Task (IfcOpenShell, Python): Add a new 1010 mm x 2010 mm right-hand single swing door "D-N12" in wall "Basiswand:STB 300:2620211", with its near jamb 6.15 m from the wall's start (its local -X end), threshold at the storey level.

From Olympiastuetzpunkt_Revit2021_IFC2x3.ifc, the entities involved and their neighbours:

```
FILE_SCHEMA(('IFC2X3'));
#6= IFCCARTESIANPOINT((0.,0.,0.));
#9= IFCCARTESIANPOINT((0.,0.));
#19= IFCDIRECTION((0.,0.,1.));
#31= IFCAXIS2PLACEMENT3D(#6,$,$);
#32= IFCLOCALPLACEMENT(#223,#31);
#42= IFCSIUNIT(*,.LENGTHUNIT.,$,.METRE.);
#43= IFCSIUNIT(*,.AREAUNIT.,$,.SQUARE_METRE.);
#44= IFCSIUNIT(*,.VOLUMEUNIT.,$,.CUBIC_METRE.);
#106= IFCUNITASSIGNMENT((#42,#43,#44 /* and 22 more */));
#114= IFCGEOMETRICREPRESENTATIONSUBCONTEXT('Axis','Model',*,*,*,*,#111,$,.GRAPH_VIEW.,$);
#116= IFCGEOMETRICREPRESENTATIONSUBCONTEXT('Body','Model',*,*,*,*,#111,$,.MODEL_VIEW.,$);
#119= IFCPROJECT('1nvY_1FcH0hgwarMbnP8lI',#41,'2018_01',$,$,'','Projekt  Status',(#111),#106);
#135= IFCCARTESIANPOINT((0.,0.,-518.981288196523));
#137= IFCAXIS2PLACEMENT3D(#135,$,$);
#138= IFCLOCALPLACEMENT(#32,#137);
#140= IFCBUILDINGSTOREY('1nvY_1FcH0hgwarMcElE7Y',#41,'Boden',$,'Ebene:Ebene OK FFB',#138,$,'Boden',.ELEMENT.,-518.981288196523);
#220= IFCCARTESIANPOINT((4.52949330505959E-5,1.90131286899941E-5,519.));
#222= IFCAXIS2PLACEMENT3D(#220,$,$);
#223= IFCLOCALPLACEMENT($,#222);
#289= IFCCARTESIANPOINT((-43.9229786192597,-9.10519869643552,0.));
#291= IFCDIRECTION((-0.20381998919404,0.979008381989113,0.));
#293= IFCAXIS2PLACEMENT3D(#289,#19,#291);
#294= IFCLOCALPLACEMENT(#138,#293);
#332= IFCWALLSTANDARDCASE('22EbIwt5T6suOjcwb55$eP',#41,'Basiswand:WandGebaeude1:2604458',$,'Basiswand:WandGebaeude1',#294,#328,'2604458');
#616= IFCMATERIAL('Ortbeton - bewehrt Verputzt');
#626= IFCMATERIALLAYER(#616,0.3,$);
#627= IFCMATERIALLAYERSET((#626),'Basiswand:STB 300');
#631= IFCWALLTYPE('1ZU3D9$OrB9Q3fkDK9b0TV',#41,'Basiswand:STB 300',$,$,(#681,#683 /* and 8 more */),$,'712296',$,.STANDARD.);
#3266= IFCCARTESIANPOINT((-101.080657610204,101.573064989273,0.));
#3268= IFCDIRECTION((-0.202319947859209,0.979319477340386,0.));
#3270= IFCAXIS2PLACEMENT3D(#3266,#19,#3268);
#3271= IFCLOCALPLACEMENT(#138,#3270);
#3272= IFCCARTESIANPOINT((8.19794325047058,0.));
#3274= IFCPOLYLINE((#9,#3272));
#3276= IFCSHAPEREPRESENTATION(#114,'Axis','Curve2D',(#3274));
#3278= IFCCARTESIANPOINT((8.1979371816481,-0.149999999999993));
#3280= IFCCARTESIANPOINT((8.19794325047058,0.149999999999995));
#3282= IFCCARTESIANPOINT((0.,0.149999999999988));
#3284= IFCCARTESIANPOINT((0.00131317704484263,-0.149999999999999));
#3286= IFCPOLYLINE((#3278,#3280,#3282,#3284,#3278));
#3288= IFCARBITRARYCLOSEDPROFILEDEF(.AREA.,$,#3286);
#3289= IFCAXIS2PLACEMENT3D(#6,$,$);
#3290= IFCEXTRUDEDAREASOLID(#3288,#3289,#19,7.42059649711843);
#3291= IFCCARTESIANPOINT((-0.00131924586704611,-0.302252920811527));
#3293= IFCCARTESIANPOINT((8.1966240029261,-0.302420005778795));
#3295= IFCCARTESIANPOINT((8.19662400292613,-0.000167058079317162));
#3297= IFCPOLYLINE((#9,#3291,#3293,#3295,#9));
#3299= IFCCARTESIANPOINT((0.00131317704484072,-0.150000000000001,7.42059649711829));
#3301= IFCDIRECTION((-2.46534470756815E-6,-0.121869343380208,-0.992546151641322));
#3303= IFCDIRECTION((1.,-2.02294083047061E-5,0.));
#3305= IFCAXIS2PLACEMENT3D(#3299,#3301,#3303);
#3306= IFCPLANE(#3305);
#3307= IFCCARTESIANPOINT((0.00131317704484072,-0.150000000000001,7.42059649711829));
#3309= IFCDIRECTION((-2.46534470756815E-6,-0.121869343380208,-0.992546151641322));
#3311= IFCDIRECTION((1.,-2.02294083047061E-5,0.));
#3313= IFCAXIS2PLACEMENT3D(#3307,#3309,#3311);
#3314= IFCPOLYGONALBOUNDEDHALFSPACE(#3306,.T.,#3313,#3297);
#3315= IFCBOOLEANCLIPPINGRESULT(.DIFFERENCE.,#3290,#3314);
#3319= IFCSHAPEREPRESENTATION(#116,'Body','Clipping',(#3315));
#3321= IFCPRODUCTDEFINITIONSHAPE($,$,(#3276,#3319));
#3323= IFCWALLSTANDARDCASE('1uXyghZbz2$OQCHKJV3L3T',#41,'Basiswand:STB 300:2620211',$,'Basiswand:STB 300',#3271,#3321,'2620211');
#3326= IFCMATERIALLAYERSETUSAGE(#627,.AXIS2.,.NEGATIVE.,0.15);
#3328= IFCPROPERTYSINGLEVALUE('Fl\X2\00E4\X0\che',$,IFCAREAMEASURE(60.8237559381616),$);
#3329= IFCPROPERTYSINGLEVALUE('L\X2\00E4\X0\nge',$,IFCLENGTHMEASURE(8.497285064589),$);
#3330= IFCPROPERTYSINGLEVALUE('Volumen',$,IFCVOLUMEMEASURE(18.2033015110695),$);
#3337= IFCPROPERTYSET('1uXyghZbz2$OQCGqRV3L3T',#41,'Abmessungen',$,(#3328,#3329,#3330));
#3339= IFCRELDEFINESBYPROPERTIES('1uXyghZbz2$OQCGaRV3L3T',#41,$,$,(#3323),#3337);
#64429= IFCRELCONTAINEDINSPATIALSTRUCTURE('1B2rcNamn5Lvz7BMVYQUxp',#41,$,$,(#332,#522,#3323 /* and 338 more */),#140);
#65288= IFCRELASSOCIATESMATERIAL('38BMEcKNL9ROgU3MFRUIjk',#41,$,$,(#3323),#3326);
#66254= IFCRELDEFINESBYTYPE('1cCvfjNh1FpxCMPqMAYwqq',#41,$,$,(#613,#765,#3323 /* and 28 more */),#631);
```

```python
import numpy as np
import ifcopenshell
import ifcopenshell.api.feature
import ifcopenshell.api.geometry
import ifcopenshell.api.pset
import ifcopenshell.api.root
import ifcopenshell.api.spatial
import ifcopenshell.api.type
import ifcopenshell.geom
import ifcopenshell.util.element
import ifcopenshell.util.placement
import ifcopenshell.util.representation
import ifcopenshell.util.shape
import ifcopenshell.util.unit

model = ifcopenshell.open("Olympiastuetzpunkt_Revit2021_IFC2x3.ifc")
unit_scale = ifcopenshell.util.unit.calculate_unit_scale(model)
area_scale = ifcopenshell.util.unit.calculate_unit_scale(model, "AREAUNIT")
volume_scale = ifcopenshell.util.unit.calculate_unit_scale(model, "VOLUMEUNIT")
settings = ifcopenshell.geom.settings()


def volume(element):
    """Net volume in cubic metres, openings subtracted."""
    shape = ifcopenshell.geom.create_shape(settings, element)
    return ifcopenshell.util.shape.get_volume(shape.geometry)


wall = model.by_guid("1uXyghZbz2$OQCHKJV3L3T")
storey = ifcopenshell.util.element.get_container(wall, ifc_class="IfcBuildingStorey")
context = ifcopenshell.util.representation.get_context(model, "Model", "Body", "MODEL_VIEW")
before = volume(wall)

width, height, from_end, sill = 1.01, 2.01, 6.15, 0.0  # metres

# The wall runs along its own X axis, and the end named is its -X end.
wall_shape = ifcopenshell.geom.create_shape(settings, wall)
x, y, z = ifcopenshell.util.shape.get_vertices(wall_shape.geometry).T
start = x.min() + from_end
face, thickness = float(y.min()), float(y.max() - y.min())
wall_matrix = ifcopenshell.util.placement.get_local_placement(wall.ObjectPlacement)
level = ifcopenshell.util.placement.get_local_placement(storey.ObjectPlacement)[2, 3]


def in_wall(x, y):
    """Placement at x, y metres in the wall's axes, at sill height."""
    matrix = wall_matrix.copy()
    matrix[:, 3] = wall_matrix @ np.array([x / unit_scale, y / unit_scale, 0.0, 1.0])
    matrix[2, 3] = level + sill / unit_scale
    return matrix


# Opening: a box that overshoots both wall faces by 50 mm.
opening = ifcopenshell.api.root.create_entity(model, ifc_class="IfcOpeningElement")
box = ifcopenshell.api.geometry.add_wall_representation(
    model, context=context, length=width, height=height, thickness=thickness + 0.1
)
ifcopenshell.api.geometry.assign_representation(model, product=opening, representation=box)
ifcopenshell.api.geometry.edit_object_placement(model, product=opening, matrix=in_wall(start, face - 0.05), is_si=False)
ifcopenshell.api.feature.add_feature(model, feature=opening, element=wall)

door = ifcopenshell.api.root.create_entity(model, ifc_class="IfcDoor", name="D-N12")
door.OverallWidth, door.OverallHeight = width / unit_scale, height / unit_scale
body = ifcopenshell.api.geometry.add_door_representation(
    model,
    context=context,
    overall_width=door.OverallWidth,
    overall_height=door.OverallHeight,
    operation_type="SINGLE_SWING_RIGHT",
    lining_properties={"LiningDepth": thickness / unit_scale, "ThresholdDepth": thickness / unit_scale},
)
ifcopenshell.api.geometry.assign_representation(model, product=door, representation=body)
ifcopenshell.api.spatial.assign_container(model, products=[door], relating_structure=storey)
fills = ifcopenshell.api.feature.add_filling(model, opening=opening, element=door)
fills.OwnerHistory = door.OwnerHistory  # required in IFC2X3

# IFC2X3 keeps the operation on the door style.
style = ifcopenshell.api.root.create_entity(model, ifc_class="IfcDoorStyle", name="D-N12")
style.OperationType, style.ConstructionType = "SINGLE_SWING_RIGHT", "NOTDEFINED"
style.ParameterTakesPrecedence = style.Sizeable = False
ifcopenshell.api.type.assign_type(model, related_objects=[door], relating_type=style)

# The lining spans the wall, so the door starts at the wall face.
ifcopenshell.api.geometry.edit_object_placement(model, product=door, matrix=in_wall(start, face), is_si=False)

after = volume(wall)

# Update the wall's stored quantities.
pset = model.by_id(ifcopenshell.util.element.get_pset(wall, "Abmessungen", should_inherit=False)["id"])
ifcopenshell.api.pset.edit_pset(model, pset=pset, properties={
    "Fläche": model.create_entity("IfcAreaMeasure", after / thickness / area_scale),
    "Volumen": model.create_entity("IfcVolumeMeasure", after / volume_scale),
})

print(f"wall volume {before:.3f} -> {after:.3f} m3")

model.write("Olympiastuetzpunkt_Revit2021_IFC2x3_v2.ifc")
```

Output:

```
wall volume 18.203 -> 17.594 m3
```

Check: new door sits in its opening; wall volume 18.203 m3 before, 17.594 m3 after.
